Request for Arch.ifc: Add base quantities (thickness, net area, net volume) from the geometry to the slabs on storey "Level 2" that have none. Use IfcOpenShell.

First a look at what the model holds.

```python
import ifcopenshell
import ifcopenshell.util.element
import ifcopenshell.util.unit

model = ifcopenshell.open("Arch.ifc")
print(model.schema)
for unit_type in ("LENGTHUNIT", "AREAUNIT", "VOLUMEUNIT"):
    print(unit_type, ifcopenshell.util.unit.calculate_unit_scale(model, unit_type))
storey = next(s for s in model.by_type("IfcBuildingStorey") if s.Name == "Level 2")
slabs = [e for e in ifcopenshell.util.element.get_decomposition(storey) if e.is_a("IfcSlab")]
for e in sorted(slabs, key=lambda e: e.id()):
    print(e.id(), e.is_a(), e.Name, list(ifcopenshell.util.element.get_psets(e, qtos_only=True)), sep=" | ")
```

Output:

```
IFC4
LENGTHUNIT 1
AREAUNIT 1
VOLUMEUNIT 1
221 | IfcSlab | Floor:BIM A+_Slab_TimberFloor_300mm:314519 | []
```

```python
import ifcopenshell
import ifcopenshell.api.pset
import ifcopenshell.geom
import ifcopenshell.util.element
import ifcopenshell.util.shape
import ifcopenshell.util.unit

model = ifcopenshell.open("Arch.ifc")
unit_scale = ifcopenshell.util.unit.calculate_unit_scale(model)
area_scale = ifcopenshell.util.unit.calculate_unit_scale(model, "AREAUNIT")
volume_scale = ifcopenshell.util.unit.calculate_unit_scale(model, "VOLUMEUNIT")
settings = ifcopenshell.geom.settings()

storey = next(s for s in model.by_type("IfcBuildingStorey") if s.Name == "Level 2")
slabs = [e for e in ifcopenshell.util.element.get_decomposition(storey) if e.is_a("IfcSlab")]

for e in sorted(slabs, key=lambda e: e.id()):
    if ifcopenshell.util.element.get_psets(e, qtos_only=True, should_inherit=False):
        continue
    # Geometry comes back in metres, in the element's own axes.
    shape = ifcopenshell.geom.create_shape(settings, e)
    values = {
        "Width": ifcopenshell.util.shape.get_z(shape.geometry) / unit_scale,
        "NetArea": ifcopenshell.util.shape.get_footprint_area(shape.geometry) / area_scale,
        "NetVolume": ifcopenshell.util.shape.get_volume(shape.geometry) / volume_scale,
    }
    qto = ifcopenshell.api.pset.add_qto(model, product=e, name="Qto_SlabBaseQuantities")
    ifcopenshell.api.pset.edit_qto(model, qto=qto, properties=values)
    print(e.id(), {k: round(v, 3) for k, v in values.items()})

model.write("Arch_rev.ifc")
```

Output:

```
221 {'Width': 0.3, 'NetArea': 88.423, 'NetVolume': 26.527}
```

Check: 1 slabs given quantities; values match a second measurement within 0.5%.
